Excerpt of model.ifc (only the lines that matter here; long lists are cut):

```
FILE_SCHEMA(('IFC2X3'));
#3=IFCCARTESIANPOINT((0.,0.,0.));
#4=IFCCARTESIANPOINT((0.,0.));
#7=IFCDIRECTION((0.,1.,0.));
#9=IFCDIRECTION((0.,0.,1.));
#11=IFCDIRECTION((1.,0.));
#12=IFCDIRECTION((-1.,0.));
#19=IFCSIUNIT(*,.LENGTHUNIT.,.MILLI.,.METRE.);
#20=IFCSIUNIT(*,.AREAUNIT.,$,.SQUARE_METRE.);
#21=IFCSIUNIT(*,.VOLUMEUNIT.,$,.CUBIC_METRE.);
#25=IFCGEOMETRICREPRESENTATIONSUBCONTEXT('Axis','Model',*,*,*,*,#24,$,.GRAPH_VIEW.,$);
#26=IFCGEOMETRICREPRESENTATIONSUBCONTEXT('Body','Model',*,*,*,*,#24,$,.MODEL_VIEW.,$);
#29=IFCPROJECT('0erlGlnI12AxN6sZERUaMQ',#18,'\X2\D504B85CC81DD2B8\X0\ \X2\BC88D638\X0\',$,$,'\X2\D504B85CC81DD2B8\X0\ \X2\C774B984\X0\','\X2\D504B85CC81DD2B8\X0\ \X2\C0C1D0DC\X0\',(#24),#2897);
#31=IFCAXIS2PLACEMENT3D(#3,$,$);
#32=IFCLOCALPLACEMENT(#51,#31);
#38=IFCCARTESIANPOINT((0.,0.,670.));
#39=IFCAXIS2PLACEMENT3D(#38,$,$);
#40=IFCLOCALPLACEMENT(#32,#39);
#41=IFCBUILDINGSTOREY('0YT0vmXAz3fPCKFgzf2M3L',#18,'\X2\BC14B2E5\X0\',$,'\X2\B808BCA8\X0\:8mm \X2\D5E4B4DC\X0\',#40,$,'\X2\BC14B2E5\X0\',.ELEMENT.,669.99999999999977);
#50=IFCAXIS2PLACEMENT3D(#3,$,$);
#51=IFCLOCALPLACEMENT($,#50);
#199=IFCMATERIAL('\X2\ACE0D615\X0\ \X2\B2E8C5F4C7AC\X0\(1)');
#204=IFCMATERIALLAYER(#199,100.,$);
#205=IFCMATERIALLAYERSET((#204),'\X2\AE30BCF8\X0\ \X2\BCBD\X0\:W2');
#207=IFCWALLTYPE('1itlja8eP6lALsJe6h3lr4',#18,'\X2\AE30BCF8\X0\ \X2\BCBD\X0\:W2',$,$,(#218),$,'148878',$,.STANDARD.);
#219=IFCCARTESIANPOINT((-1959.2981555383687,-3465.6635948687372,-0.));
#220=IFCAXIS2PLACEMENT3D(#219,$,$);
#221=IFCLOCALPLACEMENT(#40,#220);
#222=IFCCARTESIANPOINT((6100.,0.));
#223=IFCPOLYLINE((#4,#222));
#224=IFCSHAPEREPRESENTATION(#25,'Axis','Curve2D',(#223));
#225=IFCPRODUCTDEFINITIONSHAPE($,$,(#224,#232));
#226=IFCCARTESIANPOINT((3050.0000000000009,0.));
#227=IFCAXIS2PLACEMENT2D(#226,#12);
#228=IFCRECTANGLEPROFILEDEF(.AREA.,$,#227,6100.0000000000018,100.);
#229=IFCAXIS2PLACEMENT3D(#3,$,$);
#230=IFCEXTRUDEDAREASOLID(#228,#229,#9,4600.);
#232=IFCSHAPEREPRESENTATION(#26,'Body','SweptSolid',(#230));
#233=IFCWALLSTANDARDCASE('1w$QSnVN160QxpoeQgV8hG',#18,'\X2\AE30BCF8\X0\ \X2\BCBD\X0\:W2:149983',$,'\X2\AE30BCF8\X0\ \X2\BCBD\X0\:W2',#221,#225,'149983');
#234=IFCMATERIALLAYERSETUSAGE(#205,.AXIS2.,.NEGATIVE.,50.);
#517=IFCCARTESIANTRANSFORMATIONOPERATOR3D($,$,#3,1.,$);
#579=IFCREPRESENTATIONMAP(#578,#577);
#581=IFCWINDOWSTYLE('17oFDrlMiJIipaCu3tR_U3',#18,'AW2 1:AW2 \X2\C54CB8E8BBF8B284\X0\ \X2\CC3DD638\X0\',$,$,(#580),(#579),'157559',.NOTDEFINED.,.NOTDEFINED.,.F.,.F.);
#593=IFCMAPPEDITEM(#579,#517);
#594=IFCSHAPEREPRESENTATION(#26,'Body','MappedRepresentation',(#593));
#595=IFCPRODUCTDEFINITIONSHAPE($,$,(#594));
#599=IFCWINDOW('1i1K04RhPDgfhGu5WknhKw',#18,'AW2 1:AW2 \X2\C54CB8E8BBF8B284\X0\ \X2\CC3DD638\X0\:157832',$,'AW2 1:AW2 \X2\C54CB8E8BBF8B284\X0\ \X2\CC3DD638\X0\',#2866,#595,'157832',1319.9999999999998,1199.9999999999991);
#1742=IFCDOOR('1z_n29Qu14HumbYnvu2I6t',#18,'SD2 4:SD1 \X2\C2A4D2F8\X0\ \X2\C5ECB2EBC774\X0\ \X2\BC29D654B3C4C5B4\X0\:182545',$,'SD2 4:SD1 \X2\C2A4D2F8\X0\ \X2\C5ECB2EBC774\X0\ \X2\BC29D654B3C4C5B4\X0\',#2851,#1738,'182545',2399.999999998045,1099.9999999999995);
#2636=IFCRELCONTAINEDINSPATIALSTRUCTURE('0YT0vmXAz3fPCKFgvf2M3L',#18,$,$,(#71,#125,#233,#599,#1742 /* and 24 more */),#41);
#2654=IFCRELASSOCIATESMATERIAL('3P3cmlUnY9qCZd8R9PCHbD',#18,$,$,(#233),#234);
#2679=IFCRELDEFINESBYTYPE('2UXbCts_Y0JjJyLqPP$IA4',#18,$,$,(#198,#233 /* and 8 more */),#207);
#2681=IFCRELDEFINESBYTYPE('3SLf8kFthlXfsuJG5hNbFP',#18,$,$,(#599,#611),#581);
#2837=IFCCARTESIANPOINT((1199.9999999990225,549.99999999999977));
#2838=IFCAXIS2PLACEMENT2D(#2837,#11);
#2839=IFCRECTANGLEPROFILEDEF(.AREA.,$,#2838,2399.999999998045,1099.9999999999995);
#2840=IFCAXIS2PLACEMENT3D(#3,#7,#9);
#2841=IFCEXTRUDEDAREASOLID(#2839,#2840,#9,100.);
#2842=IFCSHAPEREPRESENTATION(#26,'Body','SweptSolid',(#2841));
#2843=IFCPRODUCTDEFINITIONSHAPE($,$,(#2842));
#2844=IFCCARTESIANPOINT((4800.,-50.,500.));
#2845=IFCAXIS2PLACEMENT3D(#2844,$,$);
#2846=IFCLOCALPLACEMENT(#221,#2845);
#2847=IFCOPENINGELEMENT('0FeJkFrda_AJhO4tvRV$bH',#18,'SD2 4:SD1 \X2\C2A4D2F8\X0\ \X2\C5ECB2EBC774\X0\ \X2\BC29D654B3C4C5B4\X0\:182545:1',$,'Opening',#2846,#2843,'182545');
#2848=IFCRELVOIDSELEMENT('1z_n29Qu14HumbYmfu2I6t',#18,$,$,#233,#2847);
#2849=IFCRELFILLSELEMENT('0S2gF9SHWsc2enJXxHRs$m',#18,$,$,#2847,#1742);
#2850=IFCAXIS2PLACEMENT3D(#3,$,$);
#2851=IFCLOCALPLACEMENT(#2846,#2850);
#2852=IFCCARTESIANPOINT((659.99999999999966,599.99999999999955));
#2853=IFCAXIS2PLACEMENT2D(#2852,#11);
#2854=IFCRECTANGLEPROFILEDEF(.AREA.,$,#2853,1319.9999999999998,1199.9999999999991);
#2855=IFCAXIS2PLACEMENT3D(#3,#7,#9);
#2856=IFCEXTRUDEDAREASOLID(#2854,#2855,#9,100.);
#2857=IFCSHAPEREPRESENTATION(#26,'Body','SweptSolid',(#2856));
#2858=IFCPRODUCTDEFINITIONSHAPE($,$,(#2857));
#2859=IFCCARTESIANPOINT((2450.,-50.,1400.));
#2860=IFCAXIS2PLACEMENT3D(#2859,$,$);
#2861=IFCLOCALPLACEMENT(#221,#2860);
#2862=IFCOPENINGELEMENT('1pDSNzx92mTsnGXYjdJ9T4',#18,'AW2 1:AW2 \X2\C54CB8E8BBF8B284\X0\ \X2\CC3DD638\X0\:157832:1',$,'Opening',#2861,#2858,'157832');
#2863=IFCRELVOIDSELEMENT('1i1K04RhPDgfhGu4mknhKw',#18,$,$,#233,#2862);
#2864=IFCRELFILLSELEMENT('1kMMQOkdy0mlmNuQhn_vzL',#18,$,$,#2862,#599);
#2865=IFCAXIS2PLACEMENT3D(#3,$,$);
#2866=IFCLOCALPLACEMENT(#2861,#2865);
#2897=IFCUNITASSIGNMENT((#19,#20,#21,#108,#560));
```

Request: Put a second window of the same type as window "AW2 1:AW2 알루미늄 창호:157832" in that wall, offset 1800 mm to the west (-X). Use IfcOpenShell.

```python
import ifcopenshell
import ifcopenshell.api.feature
import ifcopenshell.api.geometry
import ifcopenshell.api.root
import ifcopenshell.geom
import ifcopenshell.util.element
import ifcopenshell.util.placement
import ifcopenshell.util.shape

model = ifcopenshell.open("model.ifc")
settings = ifcopenshell.geom.settings()


def volume(element):
    """Net volume in cubic metres, openings subtracted."""
    shape = ifcopenshell.geom.create_shape(settings, element)
    return ifcopenshell.util.shape.get_volume(shape.geometry)


def reuse_history(source, copy):
    """copy_class also copies each property set's owner history, people and application; keep the originals."""
    for rel in copy.IsDefinedBy:
        if rel.is_a("IfcRelDefinesByProperties") and (history := rel.RelatingPropertyDefinition.OwnerHistory):
            rel.RelatingPropertyDefinition.OwnerHistory = source.OwnerHistory
            ifcopenshell.util.element.remove_deep2(model, history)


window = model.by_guid("1i1K04RhPDgfhGu5WknhKw")
opening = window.FillsVoids[0].RelatingOpeningElement
wall = opening.VoidsElements[0].RelatingBuildingElement
before = volume(wall)
shift = ifcopenshell.util.placement.get_local_placement(wall.ObjectPlacement)[:3, 0] * -1800.0

# copy_class copies the void relationship, type, container and properties, but no geometry.
new_opening = ifcopenshell.api.root.copy_class(model, product=opening)
new_opening.Representation = ifcopenshell.util.element.copy_deep(
    model, opening.Representation, exclude=["IfcGeometricRepresentationContext", "IfcRepresentationMap"]
)
new_opening.Name = "AW2 1:AW2 알루미늄 창호"
new_opening.Tag = None
new_window = ifcopenshell.api.root.copy_class(model, product=window)
new_window.Representation = ifcopenshell.util.element.copy_deep(
    model, window.Representation, exclude=["IfcGeometricRepresentationContext", "IfcRepresentationMap"]
)
new_window.Name = "AW2 1:AW2 알루미늄 창호"
new_window.Tag = None
reuse_history(window, new_window)
fills = ifcopenshell.api.feature.add_filling(model, opening=new_opening, element=new_window)
fills.OwnerHistory = new_window.OwnerHistory  # required in IFC2X3

for old, new in ((opening, new_opening), (window, new_window)):
    matrix = ifcopenshell.util.placement.get_local_placement(old.ObjectPlacement)
    matrix[:3, 3] += shift
    ifcopenshell.api.geometry.edit_object_placement(model, product=new, matrix=matrix, is_si=False)

after = volume(wall)

print(f"wall volume {before:.3f} -> {after:.3f} m3")

model.write("model_edited.ifc")
```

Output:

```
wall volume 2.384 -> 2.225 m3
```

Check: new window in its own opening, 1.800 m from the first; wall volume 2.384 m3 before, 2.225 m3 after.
